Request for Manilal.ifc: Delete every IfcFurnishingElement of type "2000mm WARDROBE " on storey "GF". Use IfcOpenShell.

First a look at what the model holds.

```python
import ifcopenshell
import ifcopenshell.util.element

model = ifcopenshell.open("Manilal.ifc")
print(model.schema)
storey = next(s for s in model.by_type("IfcBuildingStorey") if s.Name == "GF")
furniture = [e for e in ifcopenshell.util.element.get_decomposition(storey) if e.is_a("IfcFurnishingElement")]
seen = {}
for e in furniture:
    element_type = ifcopenshell.util.element.get_type(e)
    name = element_type.Name if element_type not in (None, e) else None
    seen[name] = seen.get(name, 0) + 1
for name, count in sorted(seen.items(), key=str):
    print(count, "x", name)
```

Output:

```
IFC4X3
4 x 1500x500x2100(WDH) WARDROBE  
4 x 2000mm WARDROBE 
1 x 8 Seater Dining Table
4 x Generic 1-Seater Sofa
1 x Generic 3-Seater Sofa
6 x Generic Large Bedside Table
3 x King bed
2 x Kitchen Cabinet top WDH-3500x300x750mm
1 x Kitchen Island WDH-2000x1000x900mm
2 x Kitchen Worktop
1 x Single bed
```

```python
import ifcopenshell
import ifcopenshell.api.root
import ifcopenshell.util.element

model = ifcopenshell.open("Manilal.ifc")

storey = next(s for s in model.by_type("IfcBuildingStorey") if s.Name == "GF")
furniture = [e for e in ifcopenshell.util.element.get_decomposition(storey) if e.is_a("IfcFurnishingElement")]
targets = [e for e in furniture if (t := ifcopenshell.util.element.get_type(e)) not in (None, e) and t.Name == "2000mm WARDROBE "]

for e in targets:
    ifcopenshell.api.root.remove_product(model, product=e)
print(len(targets), "removed")

model.write("Manilal-out.ifc")
```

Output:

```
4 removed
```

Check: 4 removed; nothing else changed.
